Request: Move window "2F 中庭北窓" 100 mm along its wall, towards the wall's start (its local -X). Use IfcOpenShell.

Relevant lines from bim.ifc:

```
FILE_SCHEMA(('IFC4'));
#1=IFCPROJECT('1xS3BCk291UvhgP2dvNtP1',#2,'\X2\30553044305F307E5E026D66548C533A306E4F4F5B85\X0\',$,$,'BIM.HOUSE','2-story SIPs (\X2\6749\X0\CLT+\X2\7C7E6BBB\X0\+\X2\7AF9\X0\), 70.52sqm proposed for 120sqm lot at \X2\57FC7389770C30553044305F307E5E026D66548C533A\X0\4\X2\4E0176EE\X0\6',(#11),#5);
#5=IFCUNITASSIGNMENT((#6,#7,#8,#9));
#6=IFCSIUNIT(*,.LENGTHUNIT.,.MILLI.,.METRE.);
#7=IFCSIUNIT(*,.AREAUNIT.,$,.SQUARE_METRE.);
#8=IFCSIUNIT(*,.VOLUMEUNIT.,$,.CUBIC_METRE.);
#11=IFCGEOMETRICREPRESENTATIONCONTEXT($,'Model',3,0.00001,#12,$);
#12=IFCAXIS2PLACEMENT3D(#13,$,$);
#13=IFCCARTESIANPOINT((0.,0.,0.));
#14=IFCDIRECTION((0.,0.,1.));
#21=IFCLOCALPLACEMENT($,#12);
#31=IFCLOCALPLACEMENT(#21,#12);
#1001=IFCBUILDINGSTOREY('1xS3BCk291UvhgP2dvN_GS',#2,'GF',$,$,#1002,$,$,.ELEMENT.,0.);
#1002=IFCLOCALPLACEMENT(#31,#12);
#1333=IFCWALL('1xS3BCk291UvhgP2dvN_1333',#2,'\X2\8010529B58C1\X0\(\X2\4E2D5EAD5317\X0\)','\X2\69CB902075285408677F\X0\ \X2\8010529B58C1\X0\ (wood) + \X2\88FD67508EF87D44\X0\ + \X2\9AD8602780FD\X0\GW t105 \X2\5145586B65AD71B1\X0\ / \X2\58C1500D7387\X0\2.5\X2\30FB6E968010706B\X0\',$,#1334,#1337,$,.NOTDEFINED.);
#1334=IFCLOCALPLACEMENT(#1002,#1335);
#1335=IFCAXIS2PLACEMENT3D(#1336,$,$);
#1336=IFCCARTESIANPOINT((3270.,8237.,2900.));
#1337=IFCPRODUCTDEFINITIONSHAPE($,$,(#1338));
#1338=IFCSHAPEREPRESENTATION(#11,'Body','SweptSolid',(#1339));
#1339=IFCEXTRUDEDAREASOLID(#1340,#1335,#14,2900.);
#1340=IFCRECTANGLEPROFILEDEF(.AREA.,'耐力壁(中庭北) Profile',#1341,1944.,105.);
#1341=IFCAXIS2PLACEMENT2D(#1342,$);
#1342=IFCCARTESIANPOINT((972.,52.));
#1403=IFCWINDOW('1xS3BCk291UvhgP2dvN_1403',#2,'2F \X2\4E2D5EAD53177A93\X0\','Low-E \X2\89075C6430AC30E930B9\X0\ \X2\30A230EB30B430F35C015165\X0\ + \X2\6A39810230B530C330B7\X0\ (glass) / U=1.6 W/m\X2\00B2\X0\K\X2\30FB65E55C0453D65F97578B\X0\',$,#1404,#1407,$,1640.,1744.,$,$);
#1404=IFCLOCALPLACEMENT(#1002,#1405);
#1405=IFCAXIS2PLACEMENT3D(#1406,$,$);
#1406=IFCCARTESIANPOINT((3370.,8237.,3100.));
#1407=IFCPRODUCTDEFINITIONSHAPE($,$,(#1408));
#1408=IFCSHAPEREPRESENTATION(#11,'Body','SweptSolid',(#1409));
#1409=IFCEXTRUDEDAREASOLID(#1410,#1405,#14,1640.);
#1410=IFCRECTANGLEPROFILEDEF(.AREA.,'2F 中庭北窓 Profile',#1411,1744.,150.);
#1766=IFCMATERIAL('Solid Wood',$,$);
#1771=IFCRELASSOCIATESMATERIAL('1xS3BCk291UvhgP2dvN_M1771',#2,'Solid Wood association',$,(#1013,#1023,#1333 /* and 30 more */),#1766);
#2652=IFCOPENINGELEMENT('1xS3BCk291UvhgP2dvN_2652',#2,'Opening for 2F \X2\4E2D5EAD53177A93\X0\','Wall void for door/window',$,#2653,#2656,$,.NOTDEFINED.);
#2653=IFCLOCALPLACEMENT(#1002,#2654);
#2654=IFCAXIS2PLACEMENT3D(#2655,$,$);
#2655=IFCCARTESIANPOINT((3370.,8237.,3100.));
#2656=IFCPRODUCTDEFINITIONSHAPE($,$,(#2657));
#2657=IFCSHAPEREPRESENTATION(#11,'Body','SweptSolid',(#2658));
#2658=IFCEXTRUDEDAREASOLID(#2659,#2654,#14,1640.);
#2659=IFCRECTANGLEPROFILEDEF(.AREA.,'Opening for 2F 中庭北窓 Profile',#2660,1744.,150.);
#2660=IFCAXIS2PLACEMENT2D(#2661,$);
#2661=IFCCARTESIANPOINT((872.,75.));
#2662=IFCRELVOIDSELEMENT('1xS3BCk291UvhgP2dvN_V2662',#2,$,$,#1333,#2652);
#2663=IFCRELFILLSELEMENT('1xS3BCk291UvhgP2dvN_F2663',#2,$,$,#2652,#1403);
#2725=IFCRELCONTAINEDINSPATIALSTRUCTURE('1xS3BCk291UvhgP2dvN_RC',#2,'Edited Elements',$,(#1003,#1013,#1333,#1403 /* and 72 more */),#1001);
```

```python
import ifcopenshell
import ifcopenshell.api.geometry
import ifcopenshell.util.placement
import ifcopenshell.util.unit

model = ifcopenshell.open("bim.ifc")
unit_scale = ifcopenshell.util.unit.calculate_unit_scale(model)

window = model.by_id(1403)
opening = window.FillsVoids[0].RelatingOpeningElement
wall = opening.VoidsElements[0].RelatingBuildingElement

wall_matrix = ifcopenshell.util.placement.get_local_placement(wall.ObjectPlacement)
shift = wall_matrix[:3, 0] * -0.1 / unit_scale
before = ifcopenshell.util.placement.get_local_placement(window.ObjectPlacement)[:3, 3].copy()

# The window is not placed relative to its opening, so move both.
for product in (opening, window):
    matrix = ifcopenshell.util.placement.get_local_placement(product.ObjectPlacement)
    matrix[:3, 3] += shift
    ifcopenshell.api.geometry.edit_object_placement(model, product=product, matrix=matrix, is_si=False)

after = ifcopenshell.util.placement.get_local_placement(window.ObjectPlacement)[:3, 3]
print("window moved by", (after - before).round(3) + 0.0)

model.write("bim_updated.ifc")
```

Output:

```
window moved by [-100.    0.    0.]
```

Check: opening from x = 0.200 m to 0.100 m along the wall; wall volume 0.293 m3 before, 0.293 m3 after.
